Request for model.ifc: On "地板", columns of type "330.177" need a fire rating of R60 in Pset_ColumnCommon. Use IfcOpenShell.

First a look at what the model holds.

```python
import ifcopenshell
import ifcopenshell.util.element

model = ifcopenshell.open("model.ifc")
print(model.schema)
storey = next(s for s in model.by_type("IfcBuildingStorey") if s.Name == "地板")
columns = [e for e in ifcopenshell.util.element.get_decomposition(storey) if e.is_a("IfcColumn")]
seen = {}
for e in columns:
    element_type = ifcopenshell.util.element.get_type(e)
    key = (element_type.Name if element_type != e and element_type else None, ifcopenshell.util.element.get_pset(e, "Pset_ColumnCommon", "FireRating"))
    seen[key] = seen.get(key, 0) + 1
for (name, value), count in sorted(seen.items(), key=str):
    print(count, "x", name, "|", value)
```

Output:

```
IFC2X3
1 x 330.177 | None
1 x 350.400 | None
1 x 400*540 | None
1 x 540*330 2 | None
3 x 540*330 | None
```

```python
import ifcopenshell
import ifcopenshell.api.pset
import ifcopenshell.util.element

model = ifcopenshell.open("model.ifc")

storey = next(s for s in model.by_type("IfcBuildingStorey") if s.Name == "地板")
columns = [e for e in ifcopenshell.util.element.get_decomposition(storey) if e.is_a("IfcColumn")]

count = 0
for e in columns:
    element_type = ifcopenshell.util.element.get_type(e)
    if element_type in (None, e) or element_type.Name != "330.177":
        continue
    # add_pset returns the element's existing set when there is one.
    pset = ifcopenshell.api.pset.add_pset(model, product=e, name="Pset_ColumnCommon")
    ifcopenshell.api.pset.edit_pset(model, pset=pset, properties={"FireRating": "R60"})
    count += 1

print(count, "columns updated")

model.write("model_updated.ifc")
```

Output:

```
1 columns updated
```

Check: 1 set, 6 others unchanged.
